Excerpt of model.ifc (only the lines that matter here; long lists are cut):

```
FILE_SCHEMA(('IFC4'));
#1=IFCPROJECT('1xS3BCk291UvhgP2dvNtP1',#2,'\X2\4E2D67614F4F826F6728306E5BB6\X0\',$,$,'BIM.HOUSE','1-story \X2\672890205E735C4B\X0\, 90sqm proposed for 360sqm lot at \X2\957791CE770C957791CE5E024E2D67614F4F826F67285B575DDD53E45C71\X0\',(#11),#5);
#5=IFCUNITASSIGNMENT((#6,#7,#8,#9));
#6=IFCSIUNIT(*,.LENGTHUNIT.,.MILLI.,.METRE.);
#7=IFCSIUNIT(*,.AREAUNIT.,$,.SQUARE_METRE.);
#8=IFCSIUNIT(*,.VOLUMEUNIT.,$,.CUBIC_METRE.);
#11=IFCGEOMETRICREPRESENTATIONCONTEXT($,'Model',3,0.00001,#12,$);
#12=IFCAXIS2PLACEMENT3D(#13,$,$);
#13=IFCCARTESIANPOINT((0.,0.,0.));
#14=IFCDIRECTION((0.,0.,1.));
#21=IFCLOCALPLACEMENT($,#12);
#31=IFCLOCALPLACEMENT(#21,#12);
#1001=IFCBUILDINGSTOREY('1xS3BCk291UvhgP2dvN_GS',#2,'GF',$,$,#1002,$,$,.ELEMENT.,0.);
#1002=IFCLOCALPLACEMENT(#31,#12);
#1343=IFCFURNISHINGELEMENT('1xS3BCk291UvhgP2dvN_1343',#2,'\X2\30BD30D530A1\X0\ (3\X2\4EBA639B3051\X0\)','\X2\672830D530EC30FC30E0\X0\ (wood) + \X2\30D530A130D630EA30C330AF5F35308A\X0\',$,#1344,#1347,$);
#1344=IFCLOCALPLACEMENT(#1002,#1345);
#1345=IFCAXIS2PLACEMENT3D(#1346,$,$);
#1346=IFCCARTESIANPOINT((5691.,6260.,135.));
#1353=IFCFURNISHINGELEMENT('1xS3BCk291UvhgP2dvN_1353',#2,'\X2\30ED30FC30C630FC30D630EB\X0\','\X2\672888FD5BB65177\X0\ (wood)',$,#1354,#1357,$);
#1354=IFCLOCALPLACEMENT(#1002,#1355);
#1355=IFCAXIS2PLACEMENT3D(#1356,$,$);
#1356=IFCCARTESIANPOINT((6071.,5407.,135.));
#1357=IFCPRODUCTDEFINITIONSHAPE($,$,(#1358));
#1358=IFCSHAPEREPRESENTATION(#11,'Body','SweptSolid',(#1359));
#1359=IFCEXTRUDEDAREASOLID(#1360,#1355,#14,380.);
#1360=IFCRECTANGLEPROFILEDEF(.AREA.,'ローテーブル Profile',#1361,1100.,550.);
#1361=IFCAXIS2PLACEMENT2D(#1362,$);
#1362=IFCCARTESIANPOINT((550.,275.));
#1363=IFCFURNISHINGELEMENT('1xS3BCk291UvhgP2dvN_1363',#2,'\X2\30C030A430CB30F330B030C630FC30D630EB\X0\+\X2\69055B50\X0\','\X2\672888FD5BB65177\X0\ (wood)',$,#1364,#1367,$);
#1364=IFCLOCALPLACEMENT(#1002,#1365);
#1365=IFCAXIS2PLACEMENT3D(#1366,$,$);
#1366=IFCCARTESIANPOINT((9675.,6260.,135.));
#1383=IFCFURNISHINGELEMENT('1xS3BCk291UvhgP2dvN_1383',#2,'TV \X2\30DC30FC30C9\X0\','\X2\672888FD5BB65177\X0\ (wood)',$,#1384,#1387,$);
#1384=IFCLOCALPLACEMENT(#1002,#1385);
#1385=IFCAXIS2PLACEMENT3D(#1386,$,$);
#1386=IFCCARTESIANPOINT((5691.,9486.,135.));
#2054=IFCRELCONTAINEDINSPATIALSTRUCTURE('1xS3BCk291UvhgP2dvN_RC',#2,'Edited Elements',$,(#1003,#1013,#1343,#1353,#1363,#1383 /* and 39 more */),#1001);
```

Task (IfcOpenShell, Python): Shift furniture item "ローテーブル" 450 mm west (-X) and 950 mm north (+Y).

```python
import ifcopenshell
import ifcopenshell.api.geometry
import ifcopenshell.util.placement

model = ifcopenshell.open("model.ifc")

item = model.by_id(1353)
matrix = ifcopenshell.util.placement.get_local_placement(item.ObjectPlacement)
matrix[0, 3] -= 450.0
matrix[1, 3] += 950.0
ifcopenshell.api.geometry.edit_object_placement(model, product=item, matrix=matrix, is_si=False)

print(ifcopenshell.util.placement.get_local_placement(item.ObjectPlacement).round(3) + 0.0)

model.write("model_updated.ifc")
```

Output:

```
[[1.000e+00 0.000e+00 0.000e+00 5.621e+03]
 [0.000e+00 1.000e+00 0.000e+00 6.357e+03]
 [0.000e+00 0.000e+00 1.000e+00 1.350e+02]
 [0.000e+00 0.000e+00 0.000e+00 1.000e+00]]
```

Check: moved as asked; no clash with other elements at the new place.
